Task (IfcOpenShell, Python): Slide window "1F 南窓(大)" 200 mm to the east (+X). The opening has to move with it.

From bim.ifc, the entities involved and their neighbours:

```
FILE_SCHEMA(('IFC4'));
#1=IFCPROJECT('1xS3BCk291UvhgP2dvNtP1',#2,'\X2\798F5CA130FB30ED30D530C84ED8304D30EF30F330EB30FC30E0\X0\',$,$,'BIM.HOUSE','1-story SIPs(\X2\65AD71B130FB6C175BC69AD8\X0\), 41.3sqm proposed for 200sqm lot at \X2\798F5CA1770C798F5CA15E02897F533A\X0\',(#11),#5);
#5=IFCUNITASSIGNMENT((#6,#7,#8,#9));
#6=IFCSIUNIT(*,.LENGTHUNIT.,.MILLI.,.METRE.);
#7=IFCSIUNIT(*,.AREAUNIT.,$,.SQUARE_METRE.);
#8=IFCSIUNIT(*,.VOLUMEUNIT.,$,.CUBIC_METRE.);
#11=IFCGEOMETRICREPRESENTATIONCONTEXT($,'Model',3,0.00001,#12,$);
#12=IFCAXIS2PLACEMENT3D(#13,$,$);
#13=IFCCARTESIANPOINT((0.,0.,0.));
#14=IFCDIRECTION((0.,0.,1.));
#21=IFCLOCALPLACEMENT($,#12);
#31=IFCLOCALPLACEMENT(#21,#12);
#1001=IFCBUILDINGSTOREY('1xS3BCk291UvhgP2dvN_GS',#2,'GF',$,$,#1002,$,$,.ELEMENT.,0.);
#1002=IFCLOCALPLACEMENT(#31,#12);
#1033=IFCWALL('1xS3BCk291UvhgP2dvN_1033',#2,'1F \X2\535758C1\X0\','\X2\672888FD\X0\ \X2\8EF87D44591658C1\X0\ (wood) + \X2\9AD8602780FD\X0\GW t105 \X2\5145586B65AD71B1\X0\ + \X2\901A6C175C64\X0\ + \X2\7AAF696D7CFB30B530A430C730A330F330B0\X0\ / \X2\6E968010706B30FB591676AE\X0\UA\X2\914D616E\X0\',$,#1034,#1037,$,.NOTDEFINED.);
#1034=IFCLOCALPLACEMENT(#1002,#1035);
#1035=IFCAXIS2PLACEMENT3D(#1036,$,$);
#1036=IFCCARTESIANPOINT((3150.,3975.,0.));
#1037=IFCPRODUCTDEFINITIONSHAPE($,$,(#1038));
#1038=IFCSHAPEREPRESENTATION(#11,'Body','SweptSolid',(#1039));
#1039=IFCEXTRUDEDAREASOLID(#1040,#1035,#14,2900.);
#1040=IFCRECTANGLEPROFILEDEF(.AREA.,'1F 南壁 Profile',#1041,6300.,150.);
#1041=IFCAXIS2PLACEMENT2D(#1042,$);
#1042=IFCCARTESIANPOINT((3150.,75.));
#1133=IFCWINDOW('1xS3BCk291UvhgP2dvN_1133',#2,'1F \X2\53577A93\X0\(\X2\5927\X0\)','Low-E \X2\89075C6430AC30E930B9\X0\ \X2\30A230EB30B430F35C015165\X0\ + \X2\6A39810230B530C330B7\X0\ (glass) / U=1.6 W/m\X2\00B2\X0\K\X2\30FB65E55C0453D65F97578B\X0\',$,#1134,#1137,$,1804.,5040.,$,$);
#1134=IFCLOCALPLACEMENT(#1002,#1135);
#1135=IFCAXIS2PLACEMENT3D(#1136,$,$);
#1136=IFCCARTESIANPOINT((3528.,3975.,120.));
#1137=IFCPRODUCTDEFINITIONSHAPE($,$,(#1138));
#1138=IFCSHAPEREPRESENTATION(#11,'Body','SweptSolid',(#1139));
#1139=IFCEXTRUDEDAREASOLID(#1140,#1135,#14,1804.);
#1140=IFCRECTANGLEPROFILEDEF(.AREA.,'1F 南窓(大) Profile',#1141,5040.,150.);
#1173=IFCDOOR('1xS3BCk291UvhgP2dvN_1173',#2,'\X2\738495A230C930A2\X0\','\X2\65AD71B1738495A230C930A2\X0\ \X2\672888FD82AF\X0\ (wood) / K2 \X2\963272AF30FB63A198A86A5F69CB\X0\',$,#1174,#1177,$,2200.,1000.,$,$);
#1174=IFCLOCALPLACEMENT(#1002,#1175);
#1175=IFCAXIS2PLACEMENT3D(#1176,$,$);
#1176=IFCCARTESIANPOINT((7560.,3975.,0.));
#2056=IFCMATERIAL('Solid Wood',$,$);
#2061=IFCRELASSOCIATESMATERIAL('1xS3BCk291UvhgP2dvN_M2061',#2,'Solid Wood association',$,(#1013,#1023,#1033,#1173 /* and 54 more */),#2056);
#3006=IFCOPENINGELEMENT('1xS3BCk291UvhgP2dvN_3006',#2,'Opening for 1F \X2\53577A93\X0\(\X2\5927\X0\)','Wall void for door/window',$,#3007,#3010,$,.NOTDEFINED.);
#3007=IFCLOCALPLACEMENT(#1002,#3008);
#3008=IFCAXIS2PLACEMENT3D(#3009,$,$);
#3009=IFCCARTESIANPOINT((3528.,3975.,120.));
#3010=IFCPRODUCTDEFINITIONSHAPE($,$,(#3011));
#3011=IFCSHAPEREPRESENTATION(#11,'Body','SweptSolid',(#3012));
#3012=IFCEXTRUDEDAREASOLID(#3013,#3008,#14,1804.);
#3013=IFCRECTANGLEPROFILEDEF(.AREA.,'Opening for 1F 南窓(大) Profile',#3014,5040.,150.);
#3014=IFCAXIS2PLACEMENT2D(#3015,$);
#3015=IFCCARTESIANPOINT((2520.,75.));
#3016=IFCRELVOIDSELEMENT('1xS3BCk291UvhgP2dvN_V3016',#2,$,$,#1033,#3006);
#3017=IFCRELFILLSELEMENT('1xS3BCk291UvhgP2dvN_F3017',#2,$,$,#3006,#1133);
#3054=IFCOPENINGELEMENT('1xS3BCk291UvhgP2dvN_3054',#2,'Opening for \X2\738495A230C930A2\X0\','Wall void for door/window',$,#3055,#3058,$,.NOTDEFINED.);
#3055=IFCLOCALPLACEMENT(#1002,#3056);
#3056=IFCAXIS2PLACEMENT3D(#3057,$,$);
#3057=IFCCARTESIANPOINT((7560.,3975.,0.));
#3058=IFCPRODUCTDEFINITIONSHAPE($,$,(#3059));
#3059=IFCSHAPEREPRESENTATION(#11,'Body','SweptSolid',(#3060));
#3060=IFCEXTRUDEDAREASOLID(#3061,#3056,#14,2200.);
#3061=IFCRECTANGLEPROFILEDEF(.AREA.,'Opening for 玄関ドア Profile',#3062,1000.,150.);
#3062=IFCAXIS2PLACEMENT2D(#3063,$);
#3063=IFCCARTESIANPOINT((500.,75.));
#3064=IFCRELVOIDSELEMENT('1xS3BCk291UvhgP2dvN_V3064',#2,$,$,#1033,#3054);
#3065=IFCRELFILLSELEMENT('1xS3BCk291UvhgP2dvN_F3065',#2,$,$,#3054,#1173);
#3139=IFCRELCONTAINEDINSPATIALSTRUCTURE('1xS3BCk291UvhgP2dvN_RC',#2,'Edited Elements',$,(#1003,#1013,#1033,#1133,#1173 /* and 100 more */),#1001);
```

```python
import ifcopenshell
import ifcopenshell.api.geometry
import ifcopenshell.util.placement
import ifcopenshell.util.unit

model = ifcopenshell.open("bim.ifc")
unit_scale = ifcopenshell.util.unit.calculate_unit_scale(model)

window = model.by_guid("1xS3BCk291UvhgP2dvN_1133")
opening = window.FillsVoids[0].RelatingOpeningElement
wall = opening.VoidsElements[0].RelatingBuildingElement

wall_matrix = ifcopenshell.util.placement.get_local_placement(wall.ObjectPlacement)
shift = wall_matrix[:3, 0] * 0.2 / unit_scale
before = ifcopenshell.util.placement.get_local_placement(window.ObjectPlacement)[:3, 3].copy()

# The window is not placed relative to its opening, so move both.
for product in (opening, window):
    matrix = ifcopenshell.util.placement.get_local_placement(product.ObjectPlacement)
    matrix[:3, 3] += shift
    ifcopenshell.api.geometry.edit_object_placement(model, product=product, matrix=matrix, is_si=False)

after = ifcopenshell.util.placement.get_local_placement(window.ObjectPlacement)[:3, 3]
print("window moved by", (after - before).round(3) + 0.0)

model.write("bim_v2.ifc")
```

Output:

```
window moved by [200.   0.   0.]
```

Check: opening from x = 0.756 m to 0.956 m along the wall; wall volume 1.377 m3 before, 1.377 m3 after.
